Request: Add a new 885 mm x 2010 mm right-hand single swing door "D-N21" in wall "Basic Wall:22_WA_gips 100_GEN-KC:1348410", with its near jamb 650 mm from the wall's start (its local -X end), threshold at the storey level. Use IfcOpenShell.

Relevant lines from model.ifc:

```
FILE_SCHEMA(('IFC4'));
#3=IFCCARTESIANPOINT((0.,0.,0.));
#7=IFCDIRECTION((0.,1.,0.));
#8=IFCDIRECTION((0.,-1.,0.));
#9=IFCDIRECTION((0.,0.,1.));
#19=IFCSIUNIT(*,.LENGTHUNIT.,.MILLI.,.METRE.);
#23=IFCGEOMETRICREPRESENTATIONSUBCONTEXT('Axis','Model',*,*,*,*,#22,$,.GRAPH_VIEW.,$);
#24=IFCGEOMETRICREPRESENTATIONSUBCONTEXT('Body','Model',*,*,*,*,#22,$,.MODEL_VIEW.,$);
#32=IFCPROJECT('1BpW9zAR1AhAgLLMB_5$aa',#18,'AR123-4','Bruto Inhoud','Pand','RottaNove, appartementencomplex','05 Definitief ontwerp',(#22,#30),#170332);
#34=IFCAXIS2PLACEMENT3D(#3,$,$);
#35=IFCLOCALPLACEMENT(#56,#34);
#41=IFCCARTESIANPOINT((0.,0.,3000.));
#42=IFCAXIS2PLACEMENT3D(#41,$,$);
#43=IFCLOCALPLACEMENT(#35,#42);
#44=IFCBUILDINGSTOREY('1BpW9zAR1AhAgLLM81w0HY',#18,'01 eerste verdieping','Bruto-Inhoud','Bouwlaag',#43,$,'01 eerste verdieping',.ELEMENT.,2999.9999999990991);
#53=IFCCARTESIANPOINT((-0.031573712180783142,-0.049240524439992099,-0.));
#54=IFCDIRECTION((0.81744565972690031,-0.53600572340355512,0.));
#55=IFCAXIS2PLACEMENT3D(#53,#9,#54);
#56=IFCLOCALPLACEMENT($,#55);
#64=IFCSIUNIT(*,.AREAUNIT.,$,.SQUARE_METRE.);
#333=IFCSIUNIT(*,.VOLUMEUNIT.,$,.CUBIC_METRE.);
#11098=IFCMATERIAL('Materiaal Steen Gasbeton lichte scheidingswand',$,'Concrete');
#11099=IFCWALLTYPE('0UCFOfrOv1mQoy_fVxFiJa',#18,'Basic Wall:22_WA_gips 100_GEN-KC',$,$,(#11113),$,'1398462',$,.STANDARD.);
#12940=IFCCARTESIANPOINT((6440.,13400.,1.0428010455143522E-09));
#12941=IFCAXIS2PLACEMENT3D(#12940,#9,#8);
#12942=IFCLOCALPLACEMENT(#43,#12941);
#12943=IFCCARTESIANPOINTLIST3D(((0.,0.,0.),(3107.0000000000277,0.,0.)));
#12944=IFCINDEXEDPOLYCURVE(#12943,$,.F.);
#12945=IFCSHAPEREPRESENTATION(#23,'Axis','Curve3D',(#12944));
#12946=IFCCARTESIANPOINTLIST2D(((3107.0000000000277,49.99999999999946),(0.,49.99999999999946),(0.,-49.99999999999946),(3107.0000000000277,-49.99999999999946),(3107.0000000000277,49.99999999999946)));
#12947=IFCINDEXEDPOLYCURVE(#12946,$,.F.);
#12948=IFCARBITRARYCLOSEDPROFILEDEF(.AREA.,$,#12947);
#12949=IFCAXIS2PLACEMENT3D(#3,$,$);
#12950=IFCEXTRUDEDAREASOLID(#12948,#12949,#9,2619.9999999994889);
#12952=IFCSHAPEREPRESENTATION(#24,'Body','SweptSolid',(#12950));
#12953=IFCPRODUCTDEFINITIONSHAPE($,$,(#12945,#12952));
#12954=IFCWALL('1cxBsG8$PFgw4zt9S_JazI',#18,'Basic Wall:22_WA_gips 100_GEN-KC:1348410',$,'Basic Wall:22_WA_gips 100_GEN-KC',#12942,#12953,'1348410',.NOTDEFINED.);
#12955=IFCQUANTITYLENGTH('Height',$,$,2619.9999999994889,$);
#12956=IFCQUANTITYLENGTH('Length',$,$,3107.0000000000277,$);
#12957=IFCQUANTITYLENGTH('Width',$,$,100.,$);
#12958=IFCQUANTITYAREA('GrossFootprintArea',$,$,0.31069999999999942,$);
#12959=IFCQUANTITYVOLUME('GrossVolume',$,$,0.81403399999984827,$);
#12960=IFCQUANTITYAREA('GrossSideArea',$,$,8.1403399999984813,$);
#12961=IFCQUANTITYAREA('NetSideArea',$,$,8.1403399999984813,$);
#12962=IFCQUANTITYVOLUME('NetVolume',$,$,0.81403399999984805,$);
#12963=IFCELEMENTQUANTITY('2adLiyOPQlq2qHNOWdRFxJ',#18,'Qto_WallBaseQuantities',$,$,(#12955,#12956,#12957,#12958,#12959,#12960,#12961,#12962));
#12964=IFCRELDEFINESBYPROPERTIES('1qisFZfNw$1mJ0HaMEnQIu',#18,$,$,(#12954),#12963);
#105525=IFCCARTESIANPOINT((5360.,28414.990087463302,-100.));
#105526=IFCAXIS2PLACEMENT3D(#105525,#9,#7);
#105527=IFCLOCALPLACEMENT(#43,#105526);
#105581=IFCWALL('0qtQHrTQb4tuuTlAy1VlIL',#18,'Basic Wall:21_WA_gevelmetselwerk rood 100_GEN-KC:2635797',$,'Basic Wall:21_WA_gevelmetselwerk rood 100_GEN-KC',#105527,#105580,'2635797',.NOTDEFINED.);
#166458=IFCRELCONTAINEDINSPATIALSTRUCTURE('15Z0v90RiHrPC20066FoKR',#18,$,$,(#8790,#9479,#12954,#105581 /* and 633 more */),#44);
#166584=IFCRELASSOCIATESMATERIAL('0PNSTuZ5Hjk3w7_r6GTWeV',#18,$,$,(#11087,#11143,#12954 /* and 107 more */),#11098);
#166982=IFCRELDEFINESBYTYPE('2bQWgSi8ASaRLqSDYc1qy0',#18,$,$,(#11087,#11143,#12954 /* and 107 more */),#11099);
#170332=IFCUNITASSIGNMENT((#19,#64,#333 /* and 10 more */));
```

```python
import numpy as np
import ifcopenshell
import ifcopenshell.api.feature
import ifcopenshell.api.geometry
import ifcopenshell.api.pset
import ifcopenshell.api.root
import ifcopenshell.api.spatial
import ifcopenshell.geom
import ifcopenshell.util.element
import ifcopenshell.util.placement
import ifcopenshell.util.representation
import ifcopenshell.util.shape
import ifcopenshell.util.unit

model = ifcopenshell.open("model.ifc")
unit_scale = ifcopenshell.util.unit.calculate_unit_scale(model)
area_scale = ifcopenshell.util.unit.calculate_unit_scale(model, "AREAUNIT")
volume_scale = ifcopenshell.util.unit.calculate_unit_scale(model, "VOLUMEUNIT")
settings = ifcopenshell.geom.settings()


def volume(element):
    """Net volume in cubic metres, openings subtracted."""
    shape = ifcopenshell.geom.create_shape(settings, element)
    return ifcopenshell.util.shape.get_volume(shape.geometry)


wall = model.by_guid("1cxBsG8$PFgw4zt9S_JazI")
storey = ifcopenshell.util.element.get_container(wall, ifc_class="IfcBuildingStorey")
context = ifcopenshell.util.representation.get_context(model, "Model", "Body", "MODEL_VIEW")
before = volume(wall)

width, height, from_end, sill = 0.885, 2.01, 0.65, 0.0  # metres

# The wall runs along its own X axis, and the end named is its -X end.
wall_shape = ifcopenshell.geom.create_shape(settings, wall)
x, y, z = ifcopenshell.util.shape.get_vertices(wall_shape.geometry).T
start = x.min() + from_end
face, thickness = float(y.min()), float(y.max() - y.min())
wall_matrix = ifcopenshell.util.placement.get_local_placement(wall.ObjectPlacement)
level = ifcopenshell.util.placement.get_local_placement(storey.ObjectPlacement)[2, 3]


def in_wall(x, y):
    """Placement at x, y metres in the wall's axes, at sill height."""
    matrix = wall_matrix.copy()
    matrix[:, 3] = wall_matrix @ np.array([x / unit_scale, y / unit_scale, 0.0, 1.0])
    matrix[2, 3] = level + sill / unit_scale
    return matrix


# Opening: a box that overshoots both wall faces by 50 mm.
opening = ifcopenshell.api.root.create_entity(model, ifc_class="IfcOpeningElement", predefined_type="OPENING")
box = ifcopenshell.api.geometry.add_wall_representation(
    model, context=context, length=width, height=height, thickness=thickness + 0.1
)
ifcopenshell.api.geometry.assign_representation(model, product=opening, representation=box)
ifcopenshell.api.geometry.edit_object_placement(model, product=opening, matrix=in_wall(start, face - 0.05), is_si=False)
ifcopenshell.api.feature.add_feature(model, feature=opening, element=wall)

door = ifcopenshell.api.root.create_entity(model, ifc_class="IfcDoor", name="D-N21", predefined_type="DOOR")
door.OverallWidth, door.OverallHeight = width / unit_scale, height / unit_scale
door.OperationType = "SINGLE_SWING_RIGHT"
body = ifcopenshell.api.geometry.add_door_representation(
    model,
    context=context,
    overall_width=door.OverallWidth,
    overall_height=door.OverallHeight,
    operation_type="SINGLE_SWING_RIGHT",
    lining_properties={"LiningDepth": thickness / unit_scale, "ThresholdDepth": thickness / unit_scale},
)
ifcopenshell.api.geometry.assign_representation(model, product=door, representation=body)
ifcopenshell.api.spatial.assign_container(model, products=[door], relating_structure=storey)
ifcopenshell.api.feature.add_filling(model, opening=opening, element=door)

# The lining spans the wall, so the door starts at the wall face.
ifcopenshell.api.geometry.edit_object_placement(model, product=door, matrix=in_wall(start, face), is_si=False)

after = volume(wall)

# Update the wall's stored quantities.
qto = model.by_id(ifcopenshell.util.element.get_pset(wall, "Qto_WallBaseQuantities", should_inherit=False)["id"])
ifcopenshell.api.pset.edit_qto(model, qto=qto, properties={
    "NetSideArea": after / thickness / area_scale,
    "NetVolume": after / volume_scale,
})

print(f"wall volume {before:.3f} -> {after:.3f} m3")

model.write("model_v2.ifc")
```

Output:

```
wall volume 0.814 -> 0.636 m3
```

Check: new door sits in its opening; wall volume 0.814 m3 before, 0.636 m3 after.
